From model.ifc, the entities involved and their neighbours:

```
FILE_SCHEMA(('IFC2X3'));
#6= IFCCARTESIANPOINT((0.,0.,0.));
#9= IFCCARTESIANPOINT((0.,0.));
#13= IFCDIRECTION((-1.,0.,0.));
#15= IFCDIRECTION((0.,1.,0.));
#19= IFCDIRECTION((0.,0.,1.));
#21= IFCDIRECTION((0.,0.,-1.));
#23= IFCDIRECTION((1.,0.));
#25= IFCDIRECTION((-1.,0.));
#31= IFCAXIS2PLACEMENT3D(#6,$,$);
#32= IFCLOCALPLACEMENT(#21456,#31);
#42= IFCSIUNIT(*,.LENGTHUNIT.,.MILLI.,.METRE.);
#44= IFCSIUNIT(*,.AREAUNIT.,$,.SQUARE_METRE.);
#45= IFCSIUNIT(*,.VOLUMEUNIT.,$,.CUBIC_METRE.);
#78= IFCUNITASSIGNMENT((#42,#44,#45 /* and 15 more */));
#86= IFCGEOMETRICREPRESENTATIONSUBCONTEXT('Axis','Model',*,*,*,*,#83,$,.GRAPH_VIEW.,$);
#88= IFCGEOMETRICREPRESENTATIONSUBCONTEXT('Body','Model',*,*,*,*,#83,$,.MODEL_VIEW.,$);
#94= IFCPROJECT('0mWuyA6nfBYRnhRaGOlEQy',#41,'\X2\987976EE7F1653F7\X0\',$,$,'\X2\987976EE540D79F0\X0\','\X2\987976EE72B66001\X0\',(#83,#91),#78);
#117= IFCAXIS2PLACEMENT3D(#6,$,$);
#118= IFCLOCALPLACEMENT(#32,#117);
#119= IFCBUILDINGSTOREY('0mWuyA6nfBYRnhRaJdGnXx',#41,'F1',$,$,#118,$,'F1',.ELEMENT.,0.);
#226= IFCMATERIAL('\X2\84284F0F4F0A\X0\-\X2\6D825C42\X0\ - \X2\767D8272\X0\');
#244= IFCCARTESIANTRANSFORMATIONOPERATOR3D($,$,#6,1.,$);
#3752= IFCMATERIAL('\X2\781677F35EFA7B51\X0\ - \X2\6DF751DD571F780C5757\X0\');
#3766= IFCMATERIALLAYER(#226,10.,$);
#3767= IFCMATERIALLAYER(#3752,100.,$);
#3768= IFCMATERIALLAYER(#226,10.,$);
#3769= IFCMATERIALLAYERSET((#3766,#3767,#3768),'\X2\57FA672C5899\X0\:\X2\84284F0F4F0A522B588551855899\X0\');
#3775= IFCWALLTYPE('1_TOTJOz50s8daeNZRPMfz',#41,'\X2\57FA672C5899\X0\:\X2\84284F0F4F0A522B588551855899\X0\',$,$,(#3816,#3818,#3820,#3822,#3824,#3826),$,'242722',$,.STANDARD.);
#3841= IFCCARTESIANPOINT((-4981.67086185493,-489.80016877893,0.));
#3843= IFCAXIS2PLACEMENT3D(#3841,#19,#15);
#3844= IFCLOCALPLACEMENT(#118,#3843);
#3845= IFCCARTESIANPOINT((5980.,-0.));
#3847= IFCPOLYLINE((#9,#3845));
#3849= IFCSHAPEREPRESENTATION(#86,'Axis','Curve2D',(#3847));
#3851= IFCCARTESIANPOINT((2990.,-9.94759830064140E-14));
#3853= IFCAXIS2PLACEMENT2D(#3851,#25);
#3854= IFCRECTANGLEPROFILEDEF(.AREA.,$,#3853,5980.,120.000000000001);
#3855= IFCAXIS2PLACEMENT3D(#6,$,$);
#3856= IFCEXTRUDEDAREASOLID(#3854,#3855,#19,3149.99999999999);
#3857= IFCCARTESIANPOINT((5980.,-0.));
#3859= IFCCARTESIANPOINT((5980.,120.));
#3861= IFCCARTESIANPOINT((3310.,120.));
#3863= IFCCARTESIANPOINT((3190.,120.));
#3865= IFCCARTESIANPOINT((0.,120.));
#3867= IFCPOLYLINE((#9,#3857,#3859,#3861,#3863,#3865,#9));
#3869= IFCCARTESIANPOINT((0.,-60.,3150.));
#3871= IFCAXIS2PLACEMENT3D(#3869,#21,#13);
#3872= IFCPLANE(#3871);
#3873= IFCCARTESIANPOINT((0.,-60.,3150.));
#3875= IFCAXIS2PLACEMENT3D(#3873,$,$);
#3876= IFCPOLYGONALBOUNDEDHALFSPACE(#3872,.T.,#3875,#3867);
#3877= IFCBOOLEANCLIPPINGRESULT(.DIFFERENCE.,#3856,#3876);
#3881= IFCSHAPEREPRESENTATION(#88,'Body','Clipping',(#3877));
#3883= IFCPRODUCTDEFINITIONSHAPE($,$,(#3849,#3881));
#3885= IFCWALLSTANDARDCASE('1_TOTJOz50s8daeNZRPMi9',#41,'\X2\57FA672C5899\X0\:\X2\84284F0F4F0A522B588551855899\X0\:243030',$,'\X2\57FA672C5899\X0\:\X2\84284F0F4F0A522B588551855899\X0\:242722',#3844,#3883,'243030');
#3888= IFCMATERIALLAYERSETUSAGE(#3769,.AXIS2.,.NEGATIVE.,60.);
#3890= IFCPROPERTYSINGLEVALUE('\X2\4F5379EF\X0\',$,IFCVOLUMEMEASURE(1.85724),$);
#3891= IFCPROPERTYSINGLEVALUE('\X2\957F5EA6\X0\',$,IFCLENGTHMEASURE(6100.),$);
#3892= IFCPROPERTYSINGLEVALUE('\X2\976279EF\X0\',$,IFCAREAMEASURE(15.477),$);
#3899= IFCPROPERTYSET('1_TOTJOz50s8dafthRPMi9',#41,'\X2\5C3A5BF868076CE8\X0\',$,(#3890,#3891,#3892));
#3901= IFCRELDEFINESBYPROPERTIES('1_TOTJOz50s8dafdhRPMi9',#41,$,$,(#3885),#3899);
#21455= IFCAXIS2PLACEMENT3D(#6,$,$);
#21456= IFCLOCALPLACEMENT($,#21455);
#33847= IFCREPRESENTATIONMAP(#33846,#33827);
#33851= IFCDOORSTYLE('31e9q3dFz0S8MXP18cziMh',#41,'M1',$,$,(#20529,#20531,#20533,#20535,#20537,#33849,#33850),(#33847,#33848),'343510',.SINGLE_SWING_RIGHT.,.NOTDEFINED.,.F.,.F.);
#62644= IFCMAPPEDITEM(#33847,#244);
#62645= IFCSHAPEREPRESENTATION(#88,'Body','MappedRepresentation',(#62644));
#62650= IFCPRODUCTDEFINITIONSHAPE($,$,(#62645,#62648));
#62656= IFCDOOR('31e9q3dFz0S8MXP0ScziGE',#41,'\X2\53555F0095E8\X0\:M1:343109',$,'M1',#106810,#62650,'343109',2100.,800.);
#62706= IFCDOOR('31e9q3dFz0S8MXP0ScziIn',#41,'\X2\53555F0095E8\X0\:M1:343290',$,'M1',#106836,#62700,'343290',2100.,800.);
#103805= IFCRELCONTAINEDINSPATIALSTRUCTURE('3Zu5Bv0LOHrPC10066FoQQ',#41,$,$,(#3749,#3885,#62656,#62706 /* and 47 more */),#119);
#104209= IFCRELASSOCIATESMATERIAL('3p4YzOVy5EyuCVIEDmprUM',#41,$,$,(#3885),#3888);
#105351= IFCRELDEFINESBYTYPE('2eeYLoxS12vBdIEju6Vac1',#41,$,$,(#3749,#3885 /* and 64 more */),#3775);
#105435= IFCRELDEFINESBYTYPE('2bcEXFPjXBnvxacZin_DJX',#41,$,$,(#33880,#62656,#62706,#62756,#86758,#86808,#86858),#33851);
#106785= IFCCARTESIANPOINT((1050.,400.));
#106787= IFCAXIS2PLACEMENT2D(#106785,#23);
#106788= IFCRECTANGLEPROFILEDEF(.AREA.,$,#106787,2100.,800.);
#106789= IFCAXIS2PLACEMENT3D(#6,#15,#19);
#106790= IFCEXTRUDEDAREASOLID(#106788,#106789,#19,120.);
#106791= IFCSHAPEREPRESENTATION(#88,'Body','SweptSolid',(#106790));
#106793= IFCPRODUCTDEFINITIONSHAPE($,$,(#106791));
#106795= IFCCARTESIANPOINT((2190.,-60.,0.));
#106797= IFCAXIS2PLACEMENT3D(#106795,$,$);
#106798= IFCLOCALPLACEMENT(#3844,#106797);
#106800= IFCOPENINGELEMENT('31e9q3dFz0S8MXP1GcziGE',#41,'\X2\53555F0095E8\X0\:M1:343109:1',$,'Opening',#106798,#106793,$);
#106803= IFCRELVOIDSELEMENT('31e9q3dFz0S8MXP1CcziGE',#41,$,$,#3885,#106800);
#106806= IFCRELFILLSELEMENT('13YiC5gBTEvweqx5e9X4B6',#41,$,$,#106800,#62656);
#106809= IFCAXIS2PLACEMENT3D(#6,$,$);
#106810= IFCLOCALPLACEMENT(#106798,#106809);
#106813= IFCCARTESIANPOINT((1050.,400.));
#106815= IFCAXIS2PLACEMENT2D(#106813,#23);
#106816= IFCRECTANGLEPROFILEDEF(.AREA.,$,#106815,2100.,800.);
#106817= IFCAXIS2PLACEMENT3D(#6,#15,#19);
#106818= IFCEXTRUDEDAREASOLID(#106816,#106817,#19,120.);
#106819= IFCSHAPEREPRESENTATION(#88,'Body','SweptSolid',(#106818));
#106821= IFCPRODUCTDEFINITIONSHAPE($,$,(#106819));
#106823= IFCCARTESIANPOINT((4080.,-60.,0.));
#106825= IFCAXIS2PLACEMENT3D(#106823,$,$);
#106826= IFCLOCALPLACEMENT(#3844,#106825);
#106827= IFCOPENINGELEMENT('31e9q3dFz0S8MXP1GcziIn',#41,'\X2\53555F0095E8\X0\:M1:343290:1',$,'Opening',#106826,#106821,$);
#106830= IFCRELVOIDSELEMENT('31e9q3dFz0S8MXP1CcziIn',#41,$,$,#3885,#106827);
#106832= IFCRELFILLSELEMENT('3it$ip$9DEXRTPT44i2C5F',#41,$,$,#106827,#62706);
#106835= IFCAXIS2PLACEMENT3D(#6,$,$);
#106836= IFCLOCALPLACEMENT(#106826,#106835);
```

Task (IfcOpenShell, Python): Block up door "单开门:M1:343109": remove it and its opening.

```python
import ifcopenshell
import ifcopenshell.api.feature
import ifcopenshell.api.pset
import ifcopenshell.api.root
import ifcopenshell.geom
import ifcopenshell.util.element
import ifcopenshell.util.shape
import ifcopenshell.util.unit

model = ifcopenshell.open("model.ifc")
area_scale = ifcopenshell.util.unit.calculate_unit_scale(model, "AREAUNIT")
volume_scale = ifcopenshell.util.unit.calculate_unit_scale(model, "VOLUMEUNIT")
settings = ifcopenshell.geom.settings()


def volume(element):
    """Net volume in cubic metres, openings subtracted."""
    shape = ifcopenshell.geom.create_shape(settings, element)
    return ifcopenshell.util.shape.get_volume(shape.geometry)


door = model.by_guid("31e9q3dFz0S8MXP0ScziGE")
opening = door.FillsVoids[0].RelatingOpeningElement
wall = opening.VoidsElements[0].RelatingBuildingElement
before = volume(wall)

ifcopenshell.api.root.remove_product(model, product=door)
ifcopenshell.api.feature.remove_feature(model, feature=opening)

after = volume(wall)
thickness = 0.12  # wall thickness in metres

# Update the wall's stored quantities.
pset = model.by_id(ifcopenshell.util.element.get_pset(wall, "尺寸标注", should_inherit=False)["id"])
ifcopenshell.api.pset.edit_pset(model, pset=pset, properties={
    "体积": model.create_entity("IfcVolumeMeasure", after / volume_scale),
    "面积": model.create_entity("IfcAreaMeasure", after / thickness / area_scale),
})

print(f"wall volume {before:.3f} -> {after:.3f} m3")

model.write("model_v2.ifc")
```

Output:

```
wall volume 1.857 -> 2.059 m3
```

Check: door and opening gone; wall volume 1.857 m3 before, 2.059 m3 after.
